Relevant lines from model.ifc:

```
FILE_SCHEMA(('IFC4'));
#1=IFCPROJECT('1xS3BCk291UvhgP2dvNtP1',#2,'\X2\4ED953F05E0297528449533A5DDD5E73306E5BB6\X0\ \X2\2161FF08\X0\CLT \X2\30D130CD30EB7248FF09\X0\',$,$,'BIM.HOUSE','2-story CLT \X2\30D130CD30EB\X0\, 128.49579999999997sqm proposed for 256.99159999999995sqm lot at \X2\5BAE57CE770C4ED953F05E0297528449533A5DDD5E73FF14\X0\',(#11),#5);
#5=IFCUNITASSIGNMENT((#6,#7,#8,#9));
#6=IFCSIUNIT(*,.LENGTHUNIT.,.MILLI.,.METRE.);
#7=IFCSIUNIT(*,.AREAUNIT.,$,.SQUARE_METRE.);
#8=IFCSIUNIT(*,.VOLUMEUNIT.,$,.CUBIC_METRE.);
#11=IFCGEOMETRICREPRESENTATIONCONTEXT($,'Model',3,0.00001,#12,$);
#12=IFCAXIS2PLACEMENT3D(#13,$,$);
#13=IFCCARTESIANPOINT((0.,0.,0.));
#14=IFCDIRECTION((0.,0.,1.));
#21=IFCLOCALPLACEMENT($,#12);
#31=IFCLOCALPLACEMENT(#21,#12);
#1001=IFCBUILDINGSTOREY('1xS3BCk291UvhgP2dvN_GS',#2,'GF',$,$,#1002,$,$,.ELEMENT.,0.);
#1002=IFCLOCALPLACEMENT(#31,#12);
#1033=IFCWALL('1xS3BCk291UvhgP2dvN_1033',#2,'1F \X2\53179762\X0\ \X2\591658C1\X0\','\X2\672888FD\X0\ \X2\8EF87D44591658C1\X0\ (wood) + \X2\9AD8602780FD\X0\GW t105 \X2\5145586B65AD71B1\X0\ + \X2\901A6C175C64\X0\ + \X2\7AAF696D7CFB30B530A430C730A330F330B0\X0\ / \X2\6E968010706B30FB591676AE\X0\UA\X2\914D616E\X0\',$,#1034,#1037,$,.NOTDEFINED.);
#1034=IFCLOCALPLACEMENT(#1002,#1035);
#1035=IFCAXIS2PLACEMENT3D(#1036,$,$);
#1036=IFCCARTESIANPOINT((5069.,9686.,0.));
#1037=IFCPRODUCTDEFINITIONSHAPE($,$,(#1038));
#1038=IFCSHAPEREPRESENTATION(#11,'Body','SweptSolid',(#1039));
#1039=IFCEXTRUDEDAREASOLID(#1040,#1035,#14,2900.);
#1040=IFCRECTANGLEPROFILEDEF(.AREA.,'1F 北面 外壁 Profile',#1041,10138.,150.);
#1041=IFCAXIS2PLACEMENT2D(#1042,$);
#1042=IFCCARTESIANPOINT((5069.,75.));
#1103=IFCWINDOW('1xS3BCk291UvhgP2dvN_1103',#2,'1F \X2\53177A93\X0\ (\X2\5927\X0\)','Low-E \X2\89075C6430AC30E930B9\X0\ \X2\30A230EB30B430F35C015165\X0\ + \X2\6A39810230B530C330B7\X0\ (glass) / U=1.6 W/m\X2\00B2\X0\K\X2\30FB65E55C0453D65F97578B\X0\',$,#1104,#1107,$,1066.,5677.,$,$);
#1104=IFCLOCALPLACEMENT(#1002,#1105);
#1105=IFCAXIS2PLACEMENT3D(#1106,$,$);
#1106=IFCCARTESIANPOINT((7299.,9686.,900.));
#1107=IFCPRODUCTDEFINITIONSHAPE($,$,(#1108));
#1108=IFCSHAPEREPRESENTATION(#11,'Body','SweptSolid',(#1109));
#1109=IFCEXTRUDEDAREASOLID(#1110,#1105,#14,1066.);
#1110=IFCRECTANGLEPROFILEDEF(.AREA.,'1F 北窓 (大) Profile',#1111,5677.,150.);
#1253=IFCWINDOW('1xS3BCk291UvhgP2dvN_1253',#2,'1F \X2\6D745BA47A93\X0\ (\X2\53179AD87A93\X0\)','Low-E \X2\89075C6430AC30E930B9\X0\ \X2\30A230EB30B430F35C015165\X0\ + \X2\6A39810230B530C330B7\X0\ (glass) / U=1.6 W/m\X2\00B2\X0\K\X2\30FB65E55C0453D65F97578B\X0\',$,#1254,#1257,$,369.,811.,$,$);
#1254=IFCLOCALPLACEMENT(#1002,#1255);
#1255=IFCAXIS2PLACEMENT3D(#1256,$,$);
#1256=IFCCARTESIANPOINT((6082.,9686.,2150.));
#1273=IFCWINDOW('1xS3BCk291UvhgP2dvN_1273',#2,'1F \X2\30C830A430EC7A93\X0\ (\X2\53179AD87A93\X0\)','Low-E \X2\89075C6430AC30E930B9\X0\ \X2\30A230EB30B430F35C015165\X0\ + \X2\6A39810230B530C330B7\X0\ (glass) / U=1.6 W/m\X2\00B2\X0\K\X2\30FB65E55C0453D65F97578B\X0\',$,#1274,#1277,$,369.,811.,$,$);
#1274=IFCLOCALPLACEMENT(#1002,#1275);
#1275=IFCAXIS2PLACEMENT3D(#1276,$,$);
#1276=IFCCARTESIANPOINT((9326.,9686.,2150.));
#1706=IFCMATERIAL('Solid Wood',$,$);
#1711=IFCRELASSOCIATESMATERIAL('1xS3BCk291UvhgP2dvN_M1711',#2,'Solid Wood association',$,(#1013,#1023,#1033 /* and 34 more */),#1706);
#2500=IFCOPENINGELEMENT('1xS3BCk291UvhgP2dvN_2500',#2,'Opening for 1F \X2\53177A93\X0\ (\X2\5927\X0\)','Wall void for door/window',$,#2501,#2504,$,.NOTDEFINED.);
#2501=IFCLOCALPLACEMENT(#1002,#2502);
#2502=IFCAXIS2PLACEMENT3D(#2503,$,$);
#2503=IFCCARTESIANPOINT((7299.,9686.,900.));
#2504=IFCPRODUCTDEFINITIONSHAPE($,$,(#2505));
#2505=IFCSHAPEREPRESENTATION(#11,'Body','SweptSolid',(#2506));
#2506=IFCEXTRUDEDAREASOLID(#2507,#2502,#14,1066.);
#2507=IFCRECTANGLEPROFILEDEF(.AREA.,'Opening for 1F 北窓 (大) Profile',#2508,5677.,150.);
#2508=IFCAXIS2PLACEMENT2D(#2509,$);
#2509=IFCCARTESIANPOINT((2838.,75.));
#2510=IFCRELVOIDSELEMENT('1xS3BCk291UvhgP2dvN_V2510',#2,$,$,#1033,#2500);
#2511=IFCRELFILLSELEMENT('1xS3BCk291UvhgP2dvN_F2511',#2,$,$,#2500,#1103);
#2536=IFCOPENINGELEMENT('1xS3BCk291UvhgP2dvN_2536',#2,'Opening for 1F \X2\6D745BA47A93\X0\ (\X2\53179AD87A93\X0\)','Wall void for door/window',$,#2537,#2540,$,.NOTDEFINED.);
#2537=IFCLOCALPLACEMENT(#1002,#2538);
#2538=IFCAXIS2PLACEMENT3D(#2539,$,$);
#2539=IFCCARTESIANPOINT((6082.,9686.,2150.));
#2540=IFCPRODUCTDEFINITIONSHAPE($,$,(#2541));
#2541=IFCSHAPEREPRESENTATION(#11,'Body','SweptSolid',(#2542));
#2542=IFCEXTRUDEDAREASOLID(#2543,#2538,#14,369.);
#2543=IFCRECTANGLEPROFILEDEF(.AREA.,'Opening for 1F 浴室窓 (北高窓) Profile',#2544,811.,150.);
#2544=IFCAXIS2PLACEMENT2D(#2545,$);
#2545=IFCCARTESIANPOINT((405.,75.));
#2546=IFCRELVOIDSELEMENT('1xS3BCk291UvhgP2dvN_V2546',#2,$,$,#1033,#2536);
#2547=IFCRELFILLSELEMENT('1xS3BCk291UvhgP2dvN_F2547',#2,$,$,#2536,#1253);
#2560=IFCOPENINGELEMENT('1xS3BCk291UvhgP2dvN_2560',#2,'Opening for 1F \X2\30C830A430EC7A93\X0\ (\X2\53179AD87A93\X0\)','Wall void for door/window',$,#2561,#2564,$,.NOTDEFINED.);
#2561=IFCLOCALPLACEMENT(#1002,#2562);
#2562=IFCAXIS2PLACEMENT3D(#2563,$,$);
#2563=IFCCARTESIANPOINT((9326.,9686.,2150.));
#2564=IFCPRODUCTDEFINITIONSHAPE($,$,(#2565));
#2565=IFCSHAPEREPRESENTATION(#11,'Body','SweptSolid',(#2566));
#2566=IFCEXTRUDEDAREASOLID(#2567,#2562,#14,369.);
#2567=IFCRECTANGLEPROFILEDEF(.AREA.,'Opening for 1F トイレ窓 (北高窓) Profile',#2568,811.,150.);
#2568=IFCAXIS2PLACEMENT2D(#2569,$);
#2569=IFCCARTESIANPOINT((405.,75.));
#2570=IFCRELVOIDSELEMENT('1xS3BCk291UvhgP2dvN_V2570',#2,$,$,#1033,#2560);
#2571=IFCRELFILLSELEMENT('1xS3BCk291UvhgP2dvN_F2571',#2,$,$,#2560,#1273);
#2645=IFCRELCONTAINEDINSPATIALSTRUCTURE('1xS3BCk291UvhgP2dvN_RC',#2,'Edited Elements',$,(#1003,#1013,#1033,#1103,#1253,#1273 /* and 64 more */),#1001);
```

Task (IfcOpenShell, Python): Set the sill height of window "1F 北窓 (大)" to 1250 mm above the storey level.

```python
import numpy as np
import ifcopenshell
import ifcopenshell.api.geometry
import ifcopenshell.geom
import ifcopenshell.util.element
import ifcopenshell.util.placement
import ifcopenshell.util.shape
import ifcopenshell.util.unit

model = ifcopenshell.open("model.ifc")
unit_scale = ifcopenshell.util.unit.calculate_unit_scale(model)

window = model.by_guid("1xS3BCk291UvhgP2dvN_1103")
opening = window.FillsVoids[0].RelatingOpeningElement
storey = ifcopenshell.util.element.get_container(window, ifc_class="IfcBuildingStorey")
level = ifcopenshell.util.placement.get_local_placement(storey.ObjectPlacement)[2, 3]

# The opening's origin need not be at the sill, so measure its lowest point.
shape = ifcopenshell.geom.create_shape(ifcopenshell.geom.settings(), opening)
bottom = ifcopenshell.util.shape.get_shape_bottom_elevation(shape, shape.geometry) / unit_scale
dz = level + 1250.0 - bottom

shift = np.array([0.0, 0.0, dz])
# The window is not placed relative to its opening, so move both.
for product in (opening, window):
    matrix = ifcopenshell.util.placement.get_local_placement(product.ObjectPlacement)
    matrix[:3, 3] += shift
    ifcopenshell.api.geometry.edit_object_placement(model, product=product, matrix=matrix, is_si=False)

print(f"moved by {dz * unit_scale:+.3f} m")

model.write("model-out.ifc")
```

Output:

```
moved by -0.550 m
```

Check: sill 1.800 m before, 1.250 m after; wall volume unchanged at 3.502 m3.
